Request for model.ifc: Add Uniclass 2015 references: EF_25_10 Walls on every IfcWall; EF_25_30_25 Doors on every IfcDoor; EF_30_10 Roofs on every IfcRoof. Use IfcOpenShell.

First a look at what the model holds.

```python
import ifcopenshell

model = ifcopenshell.open("model.ifc")
print(model.schema)
print("classifications:", [c.Name for c in model.by_type("IfcClassification")])
for ifc_class in ("IfcDoor", "IfcRoof", "IfcStair", "IfcWall", "IfcWindow"):
    print(ifc_class, len(model.by_type(ifc_class)))
```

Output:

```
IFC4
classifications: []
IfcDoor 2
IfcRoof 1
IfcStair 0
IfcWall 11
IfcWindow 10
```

```python
import ifcopenshell
import ifcopenshell.api.classification

model = ifcopenshell.open("model.ifc")

system = ifcopenshell.api.classification.add_classification(model, classification="Uniclass 2015")

codes = {
    "IfcWall": ("EF_25_10", "Walls"),
    "IfcDoor": ("EF_25_30_25", "Doors"),
    "IfcRoof": ("EF_30_10", "Roofs"),
}
for ifc_class, (code, name) in codes.items():
    products = model.by_type(ifc_class)
    ifcopenshell.api.classification.add_reference(
        model, products=products, classification=system, identification=code, name=name
    )
    print(code, len(products))

model.write("model_edited.ifc")
```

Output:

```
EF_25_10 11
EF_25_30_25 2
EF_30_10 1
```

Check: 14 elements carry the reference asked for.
